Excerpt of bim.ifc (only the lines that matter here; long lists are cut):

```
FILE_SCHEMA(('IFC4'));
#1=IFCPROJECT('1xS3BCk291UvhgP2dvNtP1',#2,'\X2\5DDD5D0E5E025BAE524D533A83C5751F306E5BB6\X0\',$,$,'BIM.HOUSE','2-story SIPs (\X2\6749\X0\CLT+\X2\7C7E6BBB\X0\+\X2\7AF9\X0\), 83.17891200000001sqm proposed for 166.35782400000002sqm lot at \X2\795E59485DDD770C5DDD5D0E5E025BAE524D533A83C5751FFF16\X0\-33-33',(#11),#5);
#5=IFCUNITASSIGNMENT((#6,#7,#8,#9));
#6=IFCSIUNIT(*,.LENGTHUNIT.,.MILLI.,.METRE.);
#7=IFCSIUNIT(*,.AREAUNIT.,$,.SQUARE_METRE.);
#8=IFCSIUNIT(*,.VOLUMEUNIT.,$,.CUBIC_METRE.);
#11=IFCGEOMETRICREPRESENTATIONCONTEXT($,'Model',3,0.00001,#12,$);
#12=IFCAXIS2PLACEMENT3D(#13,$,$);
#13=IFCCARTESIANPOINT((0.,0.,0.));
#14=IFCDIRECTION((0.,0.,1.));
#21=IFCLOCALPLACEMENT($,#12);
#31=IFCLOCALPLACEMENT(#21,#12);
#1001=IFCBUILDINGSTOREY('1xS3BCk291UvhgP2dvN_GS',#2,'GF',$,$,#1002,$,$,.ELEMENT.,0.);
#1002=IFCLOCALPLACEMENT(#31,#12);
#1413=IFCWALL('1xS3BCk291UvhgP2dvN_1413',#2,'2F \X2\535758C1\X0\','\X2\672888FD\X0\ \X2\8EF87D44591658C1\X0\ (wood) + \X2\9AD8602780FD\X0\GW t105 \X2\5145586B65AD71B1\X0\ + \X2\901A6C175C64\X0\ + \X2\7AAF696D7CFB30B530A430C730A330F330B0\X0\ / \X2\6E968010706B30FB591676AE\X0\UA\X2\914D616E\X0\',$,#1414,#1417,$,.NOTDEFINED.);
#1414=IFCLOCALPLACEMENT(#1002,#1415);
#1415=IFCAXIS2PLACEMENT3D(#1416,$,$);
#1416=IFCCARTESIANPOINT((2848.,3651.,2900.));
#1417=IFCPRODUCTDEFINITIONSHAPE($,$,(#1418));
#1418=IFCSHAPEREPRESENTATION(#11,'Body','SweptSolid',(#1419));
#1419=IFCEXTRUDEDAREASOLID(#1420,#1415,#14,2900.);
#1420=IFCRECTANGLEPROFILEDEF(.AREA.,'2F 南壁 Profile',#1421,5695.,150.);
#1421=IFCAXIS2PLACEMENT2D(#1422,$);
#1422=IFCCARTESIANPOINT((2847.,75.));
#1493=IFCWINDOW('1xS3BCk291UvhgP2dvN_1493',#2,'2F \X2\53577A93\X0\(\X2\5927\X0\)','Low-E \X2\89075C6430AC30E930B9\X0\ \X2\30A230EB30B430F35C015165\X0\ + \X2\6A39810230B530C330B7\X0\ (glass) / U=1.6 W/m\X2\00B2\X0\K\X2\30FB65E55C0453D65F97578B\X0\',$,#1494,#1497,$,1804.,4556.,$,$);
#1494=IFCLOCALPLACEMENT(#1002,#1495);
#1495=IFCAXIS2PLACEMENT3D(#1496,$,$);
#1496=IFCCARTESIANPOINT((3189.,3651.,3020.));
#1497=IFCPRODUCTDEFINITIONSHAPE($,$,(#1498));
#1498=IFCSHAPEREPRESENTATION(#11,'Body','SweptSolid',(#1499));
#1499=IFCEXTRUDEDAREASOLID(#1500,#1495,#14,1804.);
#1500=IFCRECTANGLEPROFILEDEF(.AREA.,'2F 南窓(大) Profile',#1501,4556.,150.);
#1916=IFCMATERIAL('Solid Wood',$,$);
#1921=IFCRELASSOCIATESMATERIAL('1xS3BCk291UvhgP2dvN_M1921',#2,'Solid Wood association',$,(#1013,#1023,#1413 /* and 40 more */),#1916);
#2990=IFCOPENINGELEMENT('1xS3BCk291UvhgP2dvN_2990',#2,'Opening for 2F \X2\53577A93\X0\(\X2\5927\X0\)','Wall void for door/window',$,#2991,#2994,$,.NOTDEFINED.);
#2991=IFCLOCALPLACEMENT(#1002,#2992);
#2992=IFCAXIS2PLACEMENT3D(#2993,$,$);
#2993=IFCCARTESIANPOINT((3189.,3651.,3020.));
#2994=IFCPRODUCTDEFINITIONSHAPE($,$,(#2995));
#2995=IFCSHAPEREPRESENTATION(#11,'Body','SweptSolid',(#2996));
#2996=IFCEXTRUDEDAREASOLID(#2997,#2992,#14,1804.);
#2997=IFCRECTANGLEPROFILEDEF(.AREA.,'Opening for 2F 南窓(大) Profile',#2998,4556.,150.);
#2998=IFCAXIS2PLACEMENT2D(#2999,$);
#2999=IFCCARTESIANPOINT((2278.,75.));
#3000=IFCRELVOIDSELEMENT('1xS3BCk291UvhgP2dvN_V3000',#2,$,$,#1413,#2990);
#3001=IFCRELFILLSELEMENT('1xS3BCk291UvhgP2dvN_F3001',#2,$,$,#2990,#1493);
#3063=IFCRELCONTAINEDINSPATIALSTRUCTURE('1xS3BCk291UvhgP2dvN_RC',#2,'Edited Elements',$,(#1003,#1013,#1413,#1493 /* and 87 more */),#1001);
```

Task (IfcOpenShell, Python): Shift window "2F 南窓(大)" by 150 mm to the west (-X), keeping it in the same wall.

```python
import ifcopenshell
import ifcopenshell.api.geometry
import ifcopenshell.util.placement
import ifcopenshell.util.unit

model = ifcopenshell.open("bim.ifc")
unit_scale = ifcopenshell.util.unit.calculate_unit_scale(model)

window = model.by_guid("1xS3BCk291UvhgP2dvN_1493")
opening = window.FillsVoids[0].RelatingOpeningElement
wall = opening.VoidsElements[0].RelatingBuildingElement

wall_matrix = ifcopenshell.util.placement.get_local_placement(wall.ObjectPlacement)
shift = wall_matrix[:3, 0] * -0.15 / unit_scale
before = ifcopenshell.util.placement.get_local_placement(window.ObjectPlacement)[:3, 3].copy()

# The window is not placed relative to its opening, so move both.
for product in (opening, window):
    matrix = ifcopenshell.util.placement.get_local_placement(product.ObjectPlacement)
    matrix[:3, 3] += shift
    ifcopenshell.api.geometry.edit_object_placement(model, product=product, matrix=matrix, is_si=False)

after = ifcopenshell.util.placement.get_local_placement(window.ObjectPlacement)[:3, 3]
print("window moved by", (after - before).round(3) + 0.0)

model.write("bim_updated.ifc")
```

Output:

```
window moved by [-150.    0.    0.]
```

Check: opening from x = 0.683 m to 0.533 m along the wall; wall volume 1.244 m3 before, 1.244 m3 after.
